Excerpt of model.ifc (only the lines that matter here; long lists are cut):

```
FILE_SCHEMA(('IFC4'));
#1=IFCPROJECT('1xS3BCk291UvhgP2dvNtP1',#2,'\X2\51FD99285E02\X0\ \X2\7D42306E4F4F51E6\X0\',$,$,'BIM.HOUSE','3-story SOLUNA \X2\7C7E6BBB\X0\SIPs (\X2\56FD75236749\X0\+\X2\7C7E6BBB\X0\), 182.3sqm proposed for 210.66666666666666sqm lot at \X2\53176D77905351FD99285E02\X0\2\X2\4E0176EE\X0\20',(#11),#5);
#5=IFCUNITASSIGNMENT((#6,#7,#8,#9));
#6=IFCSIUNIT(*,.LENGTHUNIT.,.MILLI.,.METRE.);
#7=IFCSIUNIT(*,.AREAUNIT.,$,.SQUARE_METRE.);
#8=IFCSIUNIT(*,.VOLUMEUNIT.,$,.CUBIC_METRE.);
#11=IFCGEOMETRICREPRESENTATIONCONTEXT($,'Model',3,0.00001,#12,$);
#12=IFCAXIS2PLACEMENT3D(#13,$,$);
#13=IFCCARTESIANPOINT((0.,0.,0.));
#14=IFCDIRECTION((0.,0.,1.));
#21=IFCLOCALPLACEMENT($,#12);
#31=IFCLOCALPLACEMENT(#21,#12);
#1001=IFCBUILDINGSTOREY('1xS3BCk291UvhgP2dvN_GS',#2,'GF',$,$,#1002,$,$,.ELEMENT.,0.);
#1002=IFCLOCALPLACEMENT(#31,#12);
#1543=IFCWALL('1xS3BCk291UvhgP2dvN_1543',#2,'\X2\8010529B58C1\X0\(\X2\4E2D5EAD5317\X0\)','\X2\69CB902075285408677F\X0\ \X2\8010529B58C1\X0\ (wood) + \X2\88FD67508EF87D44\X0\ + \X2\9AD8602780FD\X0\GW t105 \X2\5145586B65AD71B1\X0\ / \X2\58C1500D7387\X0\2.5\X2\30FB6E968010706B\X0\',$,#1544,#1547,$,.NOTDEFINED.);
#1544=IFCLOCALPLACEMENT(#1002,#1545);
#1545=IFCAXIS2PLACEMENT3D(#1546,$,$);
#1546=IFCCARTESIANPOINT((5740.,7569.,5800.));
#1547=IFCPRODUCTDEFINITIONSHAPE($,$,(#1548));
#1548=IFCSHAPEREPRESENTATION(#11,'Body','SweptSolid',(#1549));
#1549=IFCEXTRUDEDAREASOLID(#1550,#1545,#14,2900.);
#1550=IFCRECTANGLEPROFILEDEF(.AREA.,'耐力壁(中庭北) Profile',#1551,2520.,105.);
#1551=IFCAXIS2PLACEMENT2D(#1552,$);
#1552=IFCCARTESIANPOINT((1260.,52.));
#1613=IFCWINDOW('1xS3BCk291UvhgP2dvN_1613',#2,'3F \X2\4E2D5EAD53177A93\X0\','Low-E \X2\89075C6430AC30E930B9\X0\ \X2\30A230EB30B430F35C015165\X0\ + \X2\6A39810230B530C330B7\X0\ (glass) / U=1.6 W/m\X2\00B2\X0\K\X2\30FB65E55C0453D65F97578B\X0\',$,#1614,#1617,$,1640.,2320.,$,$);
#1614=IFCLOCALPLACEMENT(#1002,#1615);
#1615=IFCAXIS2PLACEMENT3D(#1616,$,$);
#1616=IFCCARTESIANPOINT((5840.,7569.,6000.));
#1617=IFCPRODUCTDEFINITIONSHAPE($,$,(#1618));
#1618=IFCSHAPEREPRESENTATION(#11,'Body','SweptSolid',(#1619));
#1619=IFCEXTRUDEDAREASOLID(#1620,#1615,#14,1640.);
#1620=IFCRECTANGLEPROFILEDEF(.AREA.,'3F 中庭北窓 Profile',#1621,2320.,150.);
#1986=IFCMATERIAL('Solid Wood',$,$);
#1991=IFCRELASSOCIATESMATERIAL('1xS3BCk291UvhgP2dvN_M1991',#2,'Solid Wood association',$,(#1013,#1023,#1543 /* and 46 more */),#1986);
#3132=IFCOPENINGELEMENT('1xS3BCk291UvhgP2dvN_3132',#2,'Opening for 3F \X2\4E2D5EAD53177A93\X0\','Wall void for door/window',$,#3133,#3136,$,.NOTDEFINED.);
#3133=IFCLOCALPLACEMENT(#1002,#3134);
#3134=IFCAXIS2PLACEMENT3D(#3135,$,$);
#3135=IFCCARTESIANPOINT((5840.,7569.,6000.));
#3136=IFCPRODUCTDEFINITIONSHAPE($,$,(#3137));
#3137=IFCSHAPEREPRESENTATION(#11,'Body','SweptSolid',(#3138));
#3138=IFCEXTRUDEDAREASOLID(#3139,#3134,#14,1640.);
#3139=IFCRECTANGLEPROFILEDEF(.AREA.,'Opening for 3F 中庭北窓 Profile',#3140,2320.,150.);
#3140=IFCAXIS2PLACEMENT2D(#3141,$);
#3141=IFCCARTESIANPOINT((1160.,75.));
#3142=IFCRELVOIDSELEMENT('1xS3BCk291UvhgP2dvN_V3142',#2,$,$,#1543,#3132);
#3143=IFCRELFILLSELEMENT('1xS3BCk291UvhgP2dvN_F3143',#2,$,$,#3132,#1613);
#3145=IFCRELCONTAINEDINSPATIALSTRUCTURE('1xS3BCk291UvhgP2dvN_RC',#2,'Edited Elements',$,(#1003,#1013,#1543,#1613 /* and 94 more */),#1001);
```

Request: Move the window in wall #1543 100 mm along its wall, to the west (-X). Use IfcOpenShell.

```python
import ifcopenshell
import ifcopenshell.api.geometry
import ifcopenshell.util.placement
import ifcopenshell.util.unit

model = ifcopenshell.open("model.ifc")
unit_scale = ifcopenshell.util.unit.calculate_unit_scale(model)

window = model.by_id(1613)
opening = window.FillsVoids[0].RelatingOpeningElement
wall = opening.VoidsElements[0].RelatingBuildingElement

wall_matrix = ifcopenshell.util.placement.get_local_placement(wall.ObjectPlacement)
shift = wall_matrix[:3, 0] * -0.1 / unit_scale
before = ifcopenshell.util.placement.get_local_placement(window.ObjectPlacement)[:3, 3].copy()

# The window is not placed relative to its opening, so move both.
for product in (opening, window):
    matrix = ifcopenshell.util.placement.get_local_placement(product.ObjectPlacement)
    matrix[:3, 3] += shift
    ifcopenshell.api.geometry.edit_object_placement(model, product=product, matrix=matrix, is_si=False)

after = ifcopenshell.util.placement.get_local_placement(window.ObjectPlacement)[:3, 3]
print("window moved by", (after - before).round(3) + 0.0)

model.write("model_rev.ifc")
```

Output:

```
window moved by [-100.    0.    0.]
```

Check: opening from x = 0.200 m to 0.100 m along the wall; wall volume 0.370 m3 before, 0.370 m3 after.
